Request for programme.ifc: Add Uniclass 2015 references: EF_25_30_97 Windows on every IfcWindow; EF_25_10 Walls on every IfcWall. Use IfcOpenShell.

First a look at what the model holds.

```python
import ifcopenshell

model = ifcopenshell.open("programme.ifc")
print(model.schema)
print("classifications:", [c.Name for c in model.by_type("IfcClassification")])
for ifc_class in ("IfcDoor", "IfcRoof", "IfcStair", "IfcWall", "IfcWindow"):
    print(ifc_class, len(model.by_type(ifc_class)))
```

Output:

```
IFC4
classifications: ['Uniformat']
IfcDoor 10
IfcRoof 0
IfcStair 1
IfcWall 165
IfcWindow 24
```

```python
import ifcopenshell
import ifcopenshell.api.classification

model = ifcopenshell.open("programme.ifc")

system = ifcopenshell.api.classification.add_classification(model, classification="Uniclass 2015")

codes = {
    "IfcWindow": ("EF_25_30_97", "Windows"),
    "IfcWall": ("EF_25_10", "Walls"),
}
for ifc_class, (code, name) in codes.items():
    products = model.by_type(ifc_class)
    ifcopenshell.api.classification.add_reference(
        model, products=products, classification=system, identification=code, name=name
    )
    print(code, len(products))

model.write("programme_v2.ifc")
```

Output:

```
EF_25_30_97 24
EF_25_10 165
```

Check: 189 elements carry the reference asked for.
